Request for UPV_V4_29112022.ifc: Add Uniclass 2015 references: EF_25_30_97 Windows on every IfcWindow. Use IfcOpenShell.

First a look at what the model holds.

```python
import ifcopenshell

model = ifcopenshell.open("UPV_V4_29112022.ifc")
print(model.schema)
print("classifications:", [c.Name for c in model.by_type("IfcClassification")])
for ifc_class in ("IfcDoor", "IfcRoof", "IfcStair", "IfcWall", "IfcWindow"):
    print(ifc_class, len(model.by_type(ifc_class)))
```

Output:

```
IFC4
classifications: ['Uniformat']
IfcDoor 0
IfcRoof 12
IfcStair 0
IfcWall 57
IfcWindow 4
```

```python
import ifcopenshell
import ifcopenshell.api.classification

model = ifcopenshell.open("UPV_V4_29112022.ifc")

system = ifcopenshell.api.classification.add_classification(model, classification="Uniclass 2015")

codes = {
    "IfcWindow": ("EF_25_30_97", "Windows"),
}
for ifc_class, (code, name) in codes.items():
    products = model.by_type(ifc_class)
    ifcopenshell.api.classification.add_reference(
        model, products=products, classification=system, identification=code, name=name
    )
    print(code, len(products))

model.write("UPV_V4_29112022_edited.ifc")
```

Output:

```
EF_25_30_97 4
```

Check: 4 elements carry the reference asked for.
